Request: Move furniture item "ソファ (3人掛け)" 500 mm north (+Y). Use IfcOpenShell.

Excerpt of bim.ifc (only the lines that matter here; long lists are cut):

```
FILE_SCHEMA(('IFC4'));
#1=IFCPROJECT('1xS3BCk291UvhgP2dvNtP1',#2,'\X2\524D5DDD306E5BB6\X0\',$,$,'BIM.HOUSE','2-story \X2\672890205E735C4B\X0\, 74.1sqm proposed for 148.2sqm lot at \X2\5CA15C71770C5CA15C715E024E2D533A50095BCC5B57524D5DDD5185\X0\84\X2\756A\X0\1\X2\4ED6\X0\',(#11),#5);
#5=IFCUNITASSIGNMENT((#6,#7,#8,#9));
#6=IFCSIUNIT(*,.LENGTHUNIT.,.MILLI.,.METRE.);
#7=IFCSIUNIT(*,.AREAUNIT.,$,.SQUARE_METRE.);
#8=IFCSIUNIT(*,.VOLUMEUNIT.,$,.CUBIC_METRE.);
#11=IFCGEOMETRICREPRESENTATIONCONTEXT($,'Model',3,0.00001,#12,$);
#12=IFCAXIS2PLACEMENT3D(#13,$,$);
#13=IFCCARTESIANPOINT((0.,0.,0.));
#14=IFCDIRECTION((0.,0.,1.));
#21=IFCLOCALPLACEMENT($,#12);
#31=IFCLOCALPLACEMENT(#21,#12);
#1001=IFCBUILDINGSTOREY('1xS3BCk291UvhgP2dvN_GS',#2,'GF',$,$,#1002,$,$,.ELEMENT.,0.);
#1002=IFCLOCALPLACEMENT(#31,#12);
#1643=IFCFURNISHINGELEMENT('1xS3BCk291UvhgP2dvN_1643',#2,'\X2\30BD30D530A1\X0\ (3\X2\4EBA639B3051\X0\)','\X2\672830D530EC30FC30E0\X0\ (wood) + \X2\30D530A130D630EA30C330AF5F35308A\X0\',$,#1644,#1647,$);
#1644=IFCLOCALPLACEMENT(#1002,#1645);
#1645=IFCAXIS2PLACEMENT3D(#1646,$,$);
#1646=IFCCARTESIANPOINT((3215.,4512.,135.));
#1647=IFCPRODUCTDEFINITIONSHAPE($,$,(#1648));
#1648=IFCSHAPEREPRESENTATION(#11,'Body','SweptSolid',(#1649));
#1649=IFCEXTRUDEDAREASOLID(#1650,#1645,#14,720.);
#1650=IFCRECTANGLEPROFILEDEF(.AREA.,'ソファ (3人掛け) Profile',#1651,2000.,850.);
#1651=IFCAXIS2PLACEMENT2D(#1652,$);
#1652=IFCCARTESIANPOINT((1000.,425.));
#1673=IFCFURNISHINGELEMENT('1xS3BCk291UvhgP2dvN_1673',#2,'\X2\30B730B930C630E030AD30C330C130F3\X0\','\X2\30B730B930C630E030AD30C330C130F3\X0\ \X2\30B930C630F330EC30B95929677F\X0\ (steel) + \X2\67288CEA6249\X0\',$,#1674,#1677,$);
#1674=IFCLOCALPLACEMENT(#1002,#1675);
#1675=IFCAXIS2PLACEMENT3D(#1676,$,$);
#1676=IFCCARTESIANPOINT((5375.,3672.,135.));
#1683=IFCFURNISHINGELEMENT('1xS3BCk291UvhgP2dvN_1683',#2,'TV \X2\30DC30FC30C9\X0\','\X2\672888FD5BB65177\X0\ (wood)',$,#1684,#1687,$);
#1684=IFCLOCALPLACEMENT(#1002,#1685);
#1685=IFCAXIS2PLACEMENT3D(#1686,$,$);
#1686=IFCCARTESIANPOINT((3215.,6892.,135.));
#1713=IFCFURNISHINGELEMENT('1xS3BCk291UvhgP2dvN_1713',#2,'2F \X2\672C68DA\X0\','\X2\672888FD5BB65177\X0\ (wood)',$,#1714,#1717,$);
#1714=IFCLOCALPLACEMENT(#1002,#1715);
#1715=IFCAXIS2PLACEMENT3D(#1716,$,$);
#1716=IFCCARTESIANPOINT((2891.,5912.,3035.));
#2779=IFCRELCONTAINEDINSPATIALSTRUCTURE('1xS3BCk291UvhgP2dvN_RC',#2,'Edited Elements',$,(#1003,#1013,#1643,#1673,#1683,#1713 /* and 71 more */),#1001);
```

```python
import ifcopenshell
import ifcopenshell.api.geometry
import ifcopenshell.util.placement
import ifcopenshell.util.unit

model = ifcopenshell.open("bim.ifc")
unit_scale = ifcopenshell.util.unit.calculate_unit_scale(model)

item = model.by_guid("1xS3BCk291UvhgP2dvN_1643")
matrix = ifcopenshell.util.placement.get_local_placement(item.ObjectPlacement)
matrix[1, 3] += 0.5 / unit_scale
ifcopenshell.api.geometry.edit_object_placement(model, product=item, matrix=matrix, is_si=False)

print(ifcopenshell.util.placement.get_local_placement(item.ObjectPlacement).round(3) + 0.0)

model.write("bim_edited.ifc")
```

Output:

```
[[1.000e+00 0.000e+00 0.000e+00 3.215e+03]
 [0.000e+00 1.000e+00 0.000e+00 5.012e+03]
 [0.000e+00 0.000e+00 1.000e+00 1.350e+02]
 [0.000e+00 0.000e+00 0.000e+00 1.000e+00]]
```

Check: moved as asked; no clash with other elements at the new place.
